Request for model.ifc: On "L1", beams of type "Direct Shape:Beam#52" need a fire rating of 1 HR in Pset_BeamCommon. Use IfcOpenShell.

First a look at what the model holds.

```python
import ifcopenshell
import ifcopenshell.util.element

model = ifcopenshell.open("model.ifc")
print(model.schema)
storey = next(s for s in model.by_type("IfcBuildingStorey") if s.Name == "L1")
beams = [e for e in ifcopenshell.util.element.get_decomposition(storey) if e.is_a("IfcBeam")]
seen = {}
for e in beams:
    element_type = ifcopenshell.util.element.get_type(e)
    key = (element_type.Name if element_type != e and element_type else None, ifcopenshell.util.element.get_pset(e, "Pset_BeamCommon", "FireRating"))
    seen[key] = seen.get(key, 0) + 1
for (name, value), count in sorted(seen.items(), key=str):
    print(count, "x", name, "|", value)
```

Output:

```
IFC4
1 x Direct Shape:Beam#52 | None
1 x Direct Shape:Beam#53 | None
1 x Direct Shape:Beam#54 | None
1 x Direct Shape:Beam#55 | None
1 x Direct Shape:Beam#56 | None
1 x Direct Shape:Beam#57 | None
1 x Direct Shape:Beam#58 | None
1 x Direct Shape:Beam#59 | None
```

```python
import ifcopenshell
import ifcopenshell.api.pset
import ifcopenshell.util.element

model = ifcopenshell.open("model.ifc")

storey = next(s for s in model.by_type("IfcBuildingStorey") if s.Name == "L1")
beams = [e for e in ifcopenshell.util.element.get_decomposition(storey) if e.is_a("IfcBeam")]

count = 0
for e in beams:
    element_type = ifcopenshell.util.element.get_type(e)
    if element_type in (None, e) or element_type.Name != "Direct Shape:Beam#52":
        continue
    # add_pset returns the element's existing set when there is one.
    pset = ifcopenshell.api.pset.add_pset(model, product=e, name="Pset_BeamCommon")
    ifcopenshell.api.pset.edit_pset(model, pset=pset, properties={"FireRating": "1 HR"})
    count += 1

print(count, "beams updated")

model.write("model-out.ifc")
```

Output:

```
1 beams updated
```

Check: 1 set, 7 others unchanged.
